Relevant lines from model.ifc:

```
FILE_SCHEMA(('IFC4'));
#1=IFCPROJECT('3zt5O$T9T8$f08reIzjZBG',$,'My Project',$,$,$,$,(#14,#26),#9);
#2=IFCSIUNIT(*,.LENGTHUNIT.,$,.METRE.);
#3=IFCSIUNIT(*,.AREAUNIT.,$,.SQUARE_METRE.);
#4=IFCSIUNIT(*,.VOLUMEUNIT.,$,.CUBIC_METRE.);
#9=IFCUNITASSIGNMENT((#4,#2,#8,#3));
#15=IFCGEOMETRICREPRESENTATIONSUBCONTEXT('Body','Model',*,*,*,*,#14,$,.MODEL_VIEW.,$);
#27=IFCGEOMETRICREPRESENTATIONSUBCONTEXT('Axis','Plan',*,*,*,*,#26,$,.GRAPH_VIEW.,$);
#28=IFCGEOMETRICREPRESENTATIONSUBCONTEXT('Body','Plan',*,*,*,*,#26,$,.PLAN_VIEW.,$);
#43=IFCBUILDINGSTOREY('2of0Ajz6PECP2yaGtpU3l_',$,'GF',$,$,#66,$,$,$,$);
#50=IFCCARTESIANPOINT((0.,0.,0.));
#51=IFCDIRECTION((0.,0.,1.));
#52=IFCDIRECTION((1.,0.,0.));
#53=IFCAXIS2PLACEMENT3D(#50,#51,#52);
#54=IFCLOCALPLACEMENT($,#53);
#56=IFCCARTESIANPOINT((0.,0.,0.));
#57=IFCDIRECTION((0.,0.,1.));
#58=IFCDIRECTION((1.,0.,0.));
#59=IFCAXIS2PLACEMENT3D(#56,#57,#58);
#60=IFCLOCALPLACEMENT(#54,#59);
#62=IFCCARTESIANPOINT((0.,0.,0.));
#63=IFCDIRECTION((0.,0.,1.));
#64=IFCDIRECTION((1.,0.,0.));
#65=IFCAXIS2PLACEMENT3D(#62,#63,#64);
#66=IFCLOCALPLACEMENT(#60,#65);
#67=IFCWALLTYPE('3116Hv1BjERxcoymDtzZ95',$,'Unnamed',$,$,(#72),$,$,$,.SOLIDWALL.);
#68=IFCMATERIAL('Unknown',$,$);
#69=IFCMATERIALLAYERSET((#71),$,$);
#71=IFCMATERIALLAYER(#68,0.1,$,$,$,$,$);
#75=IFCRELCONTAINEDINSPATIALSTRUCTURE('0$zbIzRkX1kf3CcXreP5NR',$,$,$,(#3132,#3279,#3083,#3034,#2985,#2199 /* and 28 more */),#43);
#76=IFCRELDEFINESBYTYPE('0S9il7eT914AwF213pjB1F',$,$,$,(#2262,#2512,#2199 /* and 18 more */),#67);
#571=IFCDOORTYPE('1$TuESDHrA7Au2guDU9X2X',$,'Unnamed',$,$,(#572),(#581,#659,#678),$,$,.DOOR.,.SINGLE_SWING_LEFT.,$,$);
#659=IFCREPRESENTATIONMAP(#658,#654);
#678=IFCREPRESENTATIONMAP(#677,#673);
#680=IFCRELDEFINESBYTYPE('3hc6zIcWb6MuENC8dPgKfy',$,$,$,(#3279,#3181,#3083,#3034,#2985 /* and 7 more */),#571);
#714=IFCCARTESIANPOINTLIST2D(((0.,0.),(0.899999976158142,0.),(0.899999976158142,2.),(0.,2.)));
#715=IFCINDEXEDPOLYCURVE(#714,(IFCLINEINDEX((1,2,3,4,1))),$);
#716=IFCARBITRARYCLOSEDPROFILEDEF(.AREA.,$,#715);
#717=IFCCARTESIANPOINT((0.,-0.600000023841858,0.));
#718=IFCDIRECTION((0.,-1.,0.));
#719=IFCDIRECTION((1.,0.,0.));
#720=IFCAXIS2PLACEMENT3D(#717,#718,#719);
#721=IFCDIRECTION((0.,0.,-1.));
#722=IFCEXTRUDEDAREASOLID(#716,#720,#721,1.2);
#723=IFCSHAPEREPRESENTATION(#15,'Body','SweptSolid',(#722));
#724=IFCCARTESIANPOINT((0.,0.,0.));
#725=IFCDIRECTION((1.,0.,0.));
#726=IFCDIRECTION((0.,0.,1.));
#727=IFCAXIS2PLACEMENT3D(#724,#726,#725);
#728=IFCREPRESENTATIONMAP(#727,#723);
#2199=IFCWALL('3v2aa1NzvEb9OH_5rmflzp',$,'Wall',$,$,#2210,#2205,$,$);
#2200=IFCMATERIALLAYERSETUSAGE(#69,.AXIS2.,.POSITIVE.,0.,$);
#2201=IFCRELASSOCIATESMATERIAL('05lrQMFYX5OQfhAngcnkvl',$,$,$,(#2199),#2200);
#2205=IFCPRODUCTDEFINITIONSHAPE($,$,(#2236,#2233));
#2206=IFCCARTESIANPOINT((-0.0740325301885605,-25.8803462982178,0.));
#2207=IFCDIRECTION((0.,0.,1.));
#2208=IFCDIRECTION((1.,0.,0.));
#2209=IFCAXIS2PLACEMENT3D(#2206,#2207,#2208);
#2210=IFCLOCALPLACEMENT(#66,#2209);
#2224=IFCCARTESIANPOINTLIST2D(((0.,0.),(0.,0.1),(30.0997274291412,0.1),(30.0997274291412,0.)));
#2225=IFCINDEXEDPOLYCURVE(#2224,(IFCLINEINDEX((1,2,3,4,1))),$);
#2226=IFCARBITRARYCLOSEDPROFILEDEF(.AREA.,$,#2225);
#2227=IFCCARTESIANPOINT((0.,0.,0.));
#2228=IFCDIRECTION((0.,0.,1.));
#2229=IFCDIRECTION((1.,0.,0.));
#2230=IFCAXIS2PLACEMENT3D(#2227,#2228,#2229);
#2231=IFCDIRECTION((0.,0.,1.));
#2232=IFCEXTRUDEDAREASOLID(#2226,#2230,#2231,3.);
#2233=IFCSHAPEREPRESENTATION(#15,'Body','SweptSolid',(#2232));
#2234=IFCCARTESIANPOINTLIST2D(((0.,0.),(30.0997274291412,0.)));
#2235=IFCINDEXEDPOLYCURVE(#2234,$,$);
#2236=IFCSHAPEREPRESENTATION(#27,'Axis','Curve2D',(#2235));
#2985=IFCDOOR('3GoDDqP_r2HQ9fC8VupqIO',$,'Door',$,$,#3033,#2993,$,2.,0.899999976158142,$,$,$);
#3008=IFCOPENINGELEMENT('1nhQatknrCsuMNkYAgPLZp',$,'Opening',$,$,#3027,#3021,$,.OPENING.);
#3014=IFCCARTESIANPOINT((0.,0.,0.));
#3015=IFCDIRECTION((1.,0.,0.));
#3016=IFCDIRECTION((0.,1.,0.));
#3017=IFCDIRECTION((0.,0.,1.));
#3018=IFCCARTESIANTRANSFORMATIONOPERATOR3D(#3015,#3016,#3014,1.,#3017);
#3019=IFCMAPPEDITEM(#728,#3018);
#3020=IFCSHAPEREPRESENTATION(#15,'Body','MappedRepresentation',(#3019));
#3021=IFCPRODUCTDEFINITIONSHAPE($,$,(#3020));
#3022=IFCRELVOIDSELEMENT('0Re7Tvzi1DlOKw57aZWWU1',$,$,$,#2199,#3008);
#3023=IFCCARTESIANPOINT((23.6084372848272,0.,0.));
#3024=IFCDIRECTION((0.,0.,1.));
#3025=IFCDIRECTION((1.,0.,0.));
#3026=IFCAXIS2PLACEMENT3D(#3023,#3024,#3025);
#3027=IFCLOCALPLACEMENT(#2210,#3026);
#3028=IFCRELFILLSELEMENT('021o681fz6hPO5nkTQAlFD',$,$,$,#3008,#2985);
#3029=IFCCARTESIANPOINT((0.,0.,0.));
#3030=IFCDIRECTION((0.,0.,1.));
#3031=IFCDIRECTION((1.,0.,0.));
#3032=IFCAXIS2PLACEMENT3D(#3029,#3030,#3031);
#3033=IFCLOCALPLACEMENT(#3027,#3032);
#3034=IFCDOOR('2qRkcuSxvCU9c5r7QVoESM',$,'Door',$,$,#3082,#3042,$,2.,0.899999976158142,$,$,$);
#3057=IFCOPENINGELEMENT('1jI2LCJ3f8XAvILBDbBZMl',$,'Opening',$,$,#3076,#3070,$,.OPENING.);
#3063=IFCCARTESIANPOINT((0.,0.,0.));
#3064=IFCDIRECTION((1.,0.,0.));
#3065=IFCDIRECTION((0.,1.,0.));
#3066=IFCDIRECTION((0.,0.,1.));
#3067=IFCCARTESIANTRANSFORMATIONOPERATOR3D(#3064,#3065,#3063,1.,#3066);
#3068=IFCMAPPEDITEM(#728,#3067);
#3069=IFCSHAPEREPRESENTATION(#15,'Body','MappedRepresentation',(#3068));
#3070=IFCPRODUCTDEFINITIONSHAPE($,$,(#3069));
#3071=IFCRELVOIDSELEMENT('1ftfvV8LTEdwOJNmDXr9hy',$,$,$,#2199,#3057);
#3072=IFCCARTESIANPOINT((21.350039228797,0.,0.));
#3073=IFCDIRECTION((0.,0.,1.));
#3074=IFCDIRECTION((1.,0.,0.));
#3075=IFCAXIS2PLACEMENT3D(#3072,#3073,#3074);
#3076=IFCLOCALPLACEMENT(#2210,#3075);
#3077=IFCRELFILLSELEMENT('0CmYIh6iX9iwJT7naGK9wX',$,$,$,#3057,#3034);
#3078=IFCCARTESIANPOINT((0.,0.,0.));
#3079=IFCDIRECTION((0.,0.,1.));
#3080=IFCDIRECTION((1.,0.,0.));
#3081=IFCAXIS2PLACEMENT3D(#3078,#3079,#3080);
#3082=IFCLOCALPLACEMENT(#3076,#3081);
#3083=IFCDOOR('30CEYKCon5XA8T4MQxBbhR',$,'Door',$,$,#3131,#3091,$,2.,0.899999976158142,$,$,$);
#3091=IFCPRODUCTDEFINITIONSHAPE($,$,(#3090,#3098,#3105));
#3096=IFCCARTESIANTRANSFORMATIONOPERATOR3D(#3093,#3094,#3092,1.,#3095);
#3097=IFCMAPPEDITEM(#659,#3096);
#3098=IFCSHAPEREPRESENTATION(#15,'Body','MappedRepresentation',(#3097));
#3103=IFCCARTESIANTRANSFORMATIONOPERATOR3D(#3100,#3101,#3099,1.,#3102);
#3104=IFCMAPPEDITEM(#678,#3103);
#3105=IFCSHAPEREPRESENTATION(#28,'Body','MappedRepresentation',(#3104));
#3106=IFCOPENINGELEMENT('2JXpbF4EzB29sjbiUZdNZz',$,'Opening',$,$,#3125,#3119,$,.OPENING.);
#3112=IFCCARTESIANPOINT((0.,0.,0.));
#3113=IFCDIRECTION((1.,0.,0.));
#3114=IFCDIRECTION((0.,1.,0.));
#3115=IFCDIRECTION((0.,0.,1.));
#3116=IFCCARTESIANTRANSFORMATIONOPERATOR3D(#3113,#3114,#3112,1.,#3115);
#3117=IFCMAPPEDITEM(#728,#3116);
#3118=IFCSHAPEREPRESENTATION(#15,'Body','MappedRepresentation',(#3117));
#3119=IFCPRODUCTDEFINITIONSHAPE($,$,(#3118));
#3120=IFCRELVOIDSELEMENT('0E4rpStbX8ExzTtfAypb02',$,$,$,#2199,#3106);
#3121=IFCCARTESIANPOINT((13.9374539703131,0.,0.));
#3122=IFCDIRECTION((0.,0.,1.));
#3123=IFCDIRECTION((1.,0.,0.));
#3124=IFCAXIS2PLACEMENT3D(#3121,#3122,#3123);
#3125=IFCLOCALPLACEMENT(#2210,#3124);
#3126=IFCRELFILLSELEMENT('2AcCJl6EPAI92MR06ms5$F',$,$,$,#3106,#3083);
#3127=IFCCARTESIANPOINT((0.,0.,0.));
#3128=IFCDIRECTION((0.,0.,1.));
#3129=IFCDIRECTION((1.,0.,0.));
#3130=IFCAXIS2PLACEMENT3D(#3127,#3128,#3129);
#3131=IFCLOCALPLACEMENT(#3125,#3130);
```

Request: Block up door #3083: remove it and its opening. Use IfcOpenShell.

```python
import ifcopenshell
import ifcopenshell.api.feature
import ifcopenshell.api.root
import ifcopenshell.geom
import ifcopenshell.util.shape

model = ifcopenshell.open("model.ifc")
settings = ifcopenshell.geom.settings()


def volume(element):
    """Net volume in cubic metres, openings subtracted."""
    shape = ifcopenshell.geom.create_shape(settings, element)
    return ifcopenshell.util.shape.get_volume(shape.geometry)


door = model.by_id(3083)
opening = door.FillsVoids[0].RelatingOpeningElement
wall = opening.VoidsElements[0].RelatingBuildingElement
before = volume(wall)

ifcopenshell.api.root.remove_product(model, product=door)
ifcopenshell.api.feature.remove_feature(model, feature=opening)

after = volume(wall)

print(f"wall volume {before:.3f} -> {after:.3f} m3")

model.write("model_v2.ifc")
```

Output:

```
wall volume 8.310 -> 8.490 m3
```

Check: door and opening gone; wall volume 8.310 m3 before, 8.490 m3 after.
